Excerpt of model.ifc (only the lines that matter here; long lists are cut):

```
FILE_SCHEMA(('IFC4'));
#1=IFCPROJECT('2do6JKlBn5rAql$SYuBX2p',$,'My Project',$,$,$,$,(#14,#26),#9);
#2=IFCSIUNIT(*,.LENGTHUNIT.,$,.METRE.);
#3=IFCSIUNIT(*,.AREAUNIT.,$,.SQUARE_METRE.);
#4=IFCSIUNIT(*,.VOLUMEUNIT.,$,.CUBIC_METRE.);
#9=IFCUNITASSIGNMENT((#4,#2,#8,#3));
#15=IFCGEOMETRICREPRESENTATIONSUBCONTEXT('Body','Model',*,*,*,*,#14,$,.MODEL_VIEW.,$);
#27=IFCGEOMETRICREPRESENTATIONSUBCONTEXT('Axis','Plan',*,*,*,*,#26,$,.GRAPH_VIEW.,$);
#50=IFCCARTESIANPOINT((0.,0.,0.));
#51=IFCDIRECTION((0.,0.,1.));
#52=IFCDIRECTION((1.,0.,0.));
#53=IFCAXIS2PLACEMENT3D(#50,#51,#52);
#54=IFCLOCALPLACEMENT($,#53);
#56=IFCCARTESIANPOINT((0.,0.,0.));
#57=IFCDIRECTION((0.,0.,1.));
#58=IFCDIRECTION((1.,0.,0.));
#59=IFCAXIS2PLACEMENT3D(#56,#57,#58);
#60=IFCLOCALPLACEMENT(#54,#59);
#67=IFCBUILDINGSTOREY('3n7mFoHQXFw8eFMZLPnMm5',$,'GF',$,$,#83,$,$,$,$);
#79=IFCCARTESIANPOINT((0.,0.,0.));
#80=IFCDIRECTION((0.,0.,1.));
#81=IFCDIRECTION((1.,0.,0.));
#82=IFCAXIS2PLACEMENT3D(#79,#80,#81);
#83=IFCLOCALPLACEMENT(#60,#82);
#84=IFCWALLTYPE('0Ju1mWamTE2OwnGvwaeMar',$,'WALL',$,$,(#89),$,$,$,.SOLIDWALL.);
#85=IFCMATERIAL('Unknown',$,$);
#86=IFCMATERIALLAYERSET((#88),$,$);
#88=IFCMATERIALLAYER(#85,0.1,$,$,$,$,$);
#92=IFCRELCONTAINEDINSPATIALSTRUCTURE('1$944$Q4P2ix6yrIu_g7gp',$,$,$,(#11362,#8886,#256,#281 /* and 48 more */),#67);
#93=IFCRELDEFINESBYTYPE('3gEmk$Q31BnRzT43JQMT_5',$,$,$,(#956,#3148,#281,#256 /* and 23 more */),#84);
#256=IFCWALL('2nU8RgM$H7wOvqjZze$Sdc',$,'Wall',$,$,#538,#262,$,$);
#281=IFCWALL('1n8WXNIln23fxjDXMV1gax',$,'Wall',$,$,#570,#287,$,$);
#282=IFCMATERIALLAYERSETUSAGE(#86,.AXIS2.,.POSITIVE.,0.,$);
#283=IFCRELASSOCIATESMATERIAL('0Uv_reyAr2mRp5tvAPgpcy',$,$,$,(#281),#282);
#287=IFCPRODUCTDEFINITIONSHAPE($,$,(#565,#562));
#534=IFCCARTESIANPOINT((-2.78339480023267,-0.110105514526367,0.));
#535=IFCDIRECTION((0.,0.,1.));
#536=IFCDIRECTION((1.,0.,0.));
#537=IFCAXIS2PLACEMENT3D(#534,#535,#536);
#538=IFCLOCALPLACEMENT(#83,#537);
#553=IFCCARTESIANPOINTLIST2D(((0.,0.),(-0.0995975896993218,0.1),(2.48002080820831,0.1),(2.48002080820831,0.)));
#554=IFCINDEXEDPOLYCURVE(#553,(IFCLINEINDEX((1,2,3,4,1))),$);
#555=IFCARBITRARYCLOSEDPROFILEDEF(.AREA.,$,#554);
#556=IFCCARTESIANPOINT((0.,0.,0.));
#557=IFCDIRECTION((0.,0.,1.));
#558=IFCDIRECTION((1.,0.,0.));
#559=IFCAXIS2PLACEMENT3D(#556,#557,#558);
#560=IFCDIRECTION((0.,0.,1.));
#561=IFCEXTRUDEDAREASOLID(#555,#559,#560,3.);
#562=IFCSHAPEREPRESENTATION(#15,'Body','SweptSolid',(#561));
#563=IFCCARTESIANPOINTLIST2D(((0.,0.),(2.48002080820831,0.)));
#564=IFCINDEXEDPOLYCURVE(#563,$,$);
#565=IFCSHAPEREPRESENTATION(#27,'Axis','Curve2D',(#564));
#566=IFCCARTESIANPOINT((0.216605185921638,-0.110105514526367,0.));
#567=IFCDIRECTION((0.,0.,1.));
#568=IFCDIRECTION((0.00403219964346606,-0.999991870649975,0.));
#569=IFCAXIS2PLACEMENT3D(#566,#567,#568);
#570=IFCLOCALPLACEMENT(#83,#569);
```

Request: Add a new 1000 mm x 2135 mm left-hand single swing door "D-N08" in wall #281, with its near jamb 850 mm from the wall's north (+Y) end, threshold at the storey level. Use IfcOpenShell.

```python
import numpy as np
import ifcopenshell
import ifcopenshell.api.feature
import ifcopenshell.api.geometry
import ifcopenshell.api.root
import ifcopenshell.api.spatial
import ifcopenshell.geom
import ifcopenshell.util.element
import ifcopenshell.util.placement
import ifcopenshell.util.representation
import ifcopenshell.util.shape
import ifcopenshell.util.unit

model = ifcopenshell.open("model.ifc")
unit_scale = ifcopenshell.util.unit.calculate_unit_scale(model)
settings = ifcopenshell.geom.settings()


def volume(element):
    """Net volume in cubic metres, openings subtracted."""
    shape = ifcopenshell.geom.create_shape(settings, element)
    return ifcopenshell.util.shape.get_volume(shape.geometry)


wall = model.by_guid("1n8WXNIln23fxjDXMV1gax")
storey = ifcopenshell.util.element.get_container(wall, ifc_class="IfcBuildingStorey")
context = ifcopenshell.util.representation.get_context(model, "Model", "Body", "MODEL_VIEW")
before = volume(wall)

width, height, from_end, sill = 1, 2.135, 0.85, 0.0  # metres

# The wall runs along its own X axis, and the end named is its -X end.
wall_shape = ifcopenshell.geom.create_shape(settings, wall)
x, y, z = ifcopenshell.util.shape.get_vertices(wall_shape.geometry).T
start = x.min() + from_end
face, thickness = float(y.min()), float(y.max() - y.min())
wall_matrix = ifcopenshell.util.placement.get_local_placement(wall.ObjectPlacement)
level = ifcopenshell.util.placement.get_local_placement(storey.ObjectPlacement)[2, 3]


def in_wall(x, y):
    """Placement at x, y metres in the wall's axes, at sill height."""
    matrix = wall_matrix.copy()
    matrix[:, 3] = wall_matrix @ np.array([x / unit_scale, y / unit_scale, 0.0, 1.0])
    matrix[2, 3] = level + sill / unit_scale
    return matrix


# Opening: a box that overshoots both wall faces by 50 mm.
opening = ifcopenshell.api.root.create_entity(model, ifc_class="IfcOpeningElement", predefined_type="OPENING")
box = ifcopenshell.api.geometry.add_wall_representation(
    model, context=context, length=width, height=height, thickness=thickness + 0.1
)
ifcopenshell.api.geometry.assign_representation(model, product=opening, representation=box)
ifcopenshell.api.geometry.edit_object_placement(model, product=opening, matrix=in_wall(start, face - 0.05), is_si=False)
ifcopenshell.api.feature.add_feature(model, feature=opening, element=wall)

door = ifcopenshell.api.root.create_entity(model, ifc_class="IfcDoor", name="D-N08", predefined_type="DOOR")
door.OverallWidth, door.OverallHeight = width / unit_scale, height / unit_scale
door.OperationType = "SINGLE_SWING_LEFT"
body = ifcopenshell.api.geometry.add_door_representation(
    model,
    context=context,
    overall_width=door.OverallWidth,
    overall_height=door.OverallHeight,
    operation_type="SINGLE_SWING_LEFT",
    lining_properties={"LiningDepth": thickness / unit_scale, "ThresholdDepth": thickness / unit_scale},
)
ifcopenshell.api.geometry.assign_representation(model, product=door, representation=body)
ifcopenshell.api.spatial.assign_container(model, products=[door], relating_structure=storey)
ifcopenshell.api.feature.add_filling(model, opening=opening, element=door)

# The lining spans the wall, so the door starts at the wall face.
ifcopenshell.api.geometry.edit_object_placement(model, product=door, matrix=in_wall(start, face), is_si=False)

after = volume(wall)

print(f"wall volume {before:.3f} -> {after:.3f} m3")

model.write("model_v2.ifc")
```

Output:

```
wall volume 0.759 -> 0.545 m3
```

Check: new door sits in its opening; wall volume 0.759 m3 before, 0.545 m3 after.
